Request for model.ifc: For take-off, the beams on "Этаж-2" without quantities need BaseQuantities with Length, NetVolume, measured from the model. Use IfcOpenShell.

First a look at what the model holds.

```python
import ifcopenshell
import ifcopenshell.util.element
import ifcopenshell.util.unit

model = ifcopenshell.open("model.ifc")
print(model.schema)
for unit_type in ("LENGTHUNIT", "AREAUNIT", "VOLUMEUNIT"):
    print(unit_type, ifcopenshell.util.unit.calculate_unit_scale(model, unit_type))
storey = next(s for s in model.by_type("IfcBuildingStorey") if s.Name == "Этаж-2")
beams = [e for e in ifcopenshell.util.element.get_decomposition(storey) if e.is_a("IfcBeam")]
for e in sorted(beams, key=lambda e: e.id()):
    print(e.id(), e.is_a(), e.Name, list(ifcopenshell.util.element.get_psets(e, qtos_only=True)), sep=" | ")
```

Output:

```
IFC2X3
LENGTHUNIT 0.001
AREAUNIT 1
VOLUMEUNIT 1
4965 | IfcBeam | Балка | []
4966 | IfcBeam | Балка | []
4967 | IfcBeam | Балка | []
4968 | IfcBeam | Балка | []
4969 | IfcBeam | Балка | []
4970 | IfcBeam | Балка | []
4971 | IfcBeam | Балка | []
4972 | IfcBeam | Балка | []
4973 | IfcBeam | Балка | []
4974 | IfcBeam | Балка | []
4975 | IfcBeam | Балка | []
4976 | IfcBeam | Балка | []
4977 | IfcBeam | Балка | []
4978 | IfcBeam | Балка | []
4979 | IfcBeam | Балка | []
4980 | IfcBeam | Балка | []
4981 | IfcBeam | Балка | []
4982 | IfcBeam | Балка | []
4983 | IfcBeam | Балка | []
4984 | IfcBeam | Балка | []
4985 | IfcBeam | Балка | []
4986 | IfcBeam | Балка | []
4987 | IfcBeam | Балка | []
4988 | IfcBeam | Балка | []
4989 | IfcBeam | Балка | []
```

```python
import ifcopenshell
import ifcopenshell.api.pset
import ifcopenshell.geom
import ifcopenshell.util.element
import ifcopenshell.util.shape
import ifcopenshell.util.unit

model = ifcopenshell.open("model.ifc")
unit_scale = ifcopenshell.util.unit.calculate_unit_scale(model)
volume_scale = ifcopenshell.util.unit.calculate_unit_scale(model, "VOLUMEUNIT")
settings = ifcopenshell.geom.settings()

storey = next(s for s in model.by_type("IfcBuildingStorey") if s.Name == "Этаж-2")
beams = [e for e in ifcopenshell.util.element.get_decomposition(storey) if e.is_a("IfcBeam")]

for e in sorted(beams, key=lambda e: e.id()):
    if ifcopenshell.util.element.get_psets(e, qtos_only=True, should_inherit=False):
        continue
    # Geometry comes back in metres, in the element's own axes.
    shape = ifcopenshell.geom.create_shape(settings, e)
    values = {
        "Length": ifcopenshell.util.shape.get_max_xyz(shape.geometry) / unit_scale,
        "NetVolume": ifcopenshell.util.shape.get_volume(shape.geometry) / volume_scale,
    }
    qto = ifcopenshell.api.pset.add_qto(model, product=e, name="BaseQuantities")
    ifcopenshell.api.pset.edit_qto(model, qto=qto, properties=values)
    print(e.id(), {k: round(v, 3) for k, v in values.items()})

model.write("model-out.ifc")
```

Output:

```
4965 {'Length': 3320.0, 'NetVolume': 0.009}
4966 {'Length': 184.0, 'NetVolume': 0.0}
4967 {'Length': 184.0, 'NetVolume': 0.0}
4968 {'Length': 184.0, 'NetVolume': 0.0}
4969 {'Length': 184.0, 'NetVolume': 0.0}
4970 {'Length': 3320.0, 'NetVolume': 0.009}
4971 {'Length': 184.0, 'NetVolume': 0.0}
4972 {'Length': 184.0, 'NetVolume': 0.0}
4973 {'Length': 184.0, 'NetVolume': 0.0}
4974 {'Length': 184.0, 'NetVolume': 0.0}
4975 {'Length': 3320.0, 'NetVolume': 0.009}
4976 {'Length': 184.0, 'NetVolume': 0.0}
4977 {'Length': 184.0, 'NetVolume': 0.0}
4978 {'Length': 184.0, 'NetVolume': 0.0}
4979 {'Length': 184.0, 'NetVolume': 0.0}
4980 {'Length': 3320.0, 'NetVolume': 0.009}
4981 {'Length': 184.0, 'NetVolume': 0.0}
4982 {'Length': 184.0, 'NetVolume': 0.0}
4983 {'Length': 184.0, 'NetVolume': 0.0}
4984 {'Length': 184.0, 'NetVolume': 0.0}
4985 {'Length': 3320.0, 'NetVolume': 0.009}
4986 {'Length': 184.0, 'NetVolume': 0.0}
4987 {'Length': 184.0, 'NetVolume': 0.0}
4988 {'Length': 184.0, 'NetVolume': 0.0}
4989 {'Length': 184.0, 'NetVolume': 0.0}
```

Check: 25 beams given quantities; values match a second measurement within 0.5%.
